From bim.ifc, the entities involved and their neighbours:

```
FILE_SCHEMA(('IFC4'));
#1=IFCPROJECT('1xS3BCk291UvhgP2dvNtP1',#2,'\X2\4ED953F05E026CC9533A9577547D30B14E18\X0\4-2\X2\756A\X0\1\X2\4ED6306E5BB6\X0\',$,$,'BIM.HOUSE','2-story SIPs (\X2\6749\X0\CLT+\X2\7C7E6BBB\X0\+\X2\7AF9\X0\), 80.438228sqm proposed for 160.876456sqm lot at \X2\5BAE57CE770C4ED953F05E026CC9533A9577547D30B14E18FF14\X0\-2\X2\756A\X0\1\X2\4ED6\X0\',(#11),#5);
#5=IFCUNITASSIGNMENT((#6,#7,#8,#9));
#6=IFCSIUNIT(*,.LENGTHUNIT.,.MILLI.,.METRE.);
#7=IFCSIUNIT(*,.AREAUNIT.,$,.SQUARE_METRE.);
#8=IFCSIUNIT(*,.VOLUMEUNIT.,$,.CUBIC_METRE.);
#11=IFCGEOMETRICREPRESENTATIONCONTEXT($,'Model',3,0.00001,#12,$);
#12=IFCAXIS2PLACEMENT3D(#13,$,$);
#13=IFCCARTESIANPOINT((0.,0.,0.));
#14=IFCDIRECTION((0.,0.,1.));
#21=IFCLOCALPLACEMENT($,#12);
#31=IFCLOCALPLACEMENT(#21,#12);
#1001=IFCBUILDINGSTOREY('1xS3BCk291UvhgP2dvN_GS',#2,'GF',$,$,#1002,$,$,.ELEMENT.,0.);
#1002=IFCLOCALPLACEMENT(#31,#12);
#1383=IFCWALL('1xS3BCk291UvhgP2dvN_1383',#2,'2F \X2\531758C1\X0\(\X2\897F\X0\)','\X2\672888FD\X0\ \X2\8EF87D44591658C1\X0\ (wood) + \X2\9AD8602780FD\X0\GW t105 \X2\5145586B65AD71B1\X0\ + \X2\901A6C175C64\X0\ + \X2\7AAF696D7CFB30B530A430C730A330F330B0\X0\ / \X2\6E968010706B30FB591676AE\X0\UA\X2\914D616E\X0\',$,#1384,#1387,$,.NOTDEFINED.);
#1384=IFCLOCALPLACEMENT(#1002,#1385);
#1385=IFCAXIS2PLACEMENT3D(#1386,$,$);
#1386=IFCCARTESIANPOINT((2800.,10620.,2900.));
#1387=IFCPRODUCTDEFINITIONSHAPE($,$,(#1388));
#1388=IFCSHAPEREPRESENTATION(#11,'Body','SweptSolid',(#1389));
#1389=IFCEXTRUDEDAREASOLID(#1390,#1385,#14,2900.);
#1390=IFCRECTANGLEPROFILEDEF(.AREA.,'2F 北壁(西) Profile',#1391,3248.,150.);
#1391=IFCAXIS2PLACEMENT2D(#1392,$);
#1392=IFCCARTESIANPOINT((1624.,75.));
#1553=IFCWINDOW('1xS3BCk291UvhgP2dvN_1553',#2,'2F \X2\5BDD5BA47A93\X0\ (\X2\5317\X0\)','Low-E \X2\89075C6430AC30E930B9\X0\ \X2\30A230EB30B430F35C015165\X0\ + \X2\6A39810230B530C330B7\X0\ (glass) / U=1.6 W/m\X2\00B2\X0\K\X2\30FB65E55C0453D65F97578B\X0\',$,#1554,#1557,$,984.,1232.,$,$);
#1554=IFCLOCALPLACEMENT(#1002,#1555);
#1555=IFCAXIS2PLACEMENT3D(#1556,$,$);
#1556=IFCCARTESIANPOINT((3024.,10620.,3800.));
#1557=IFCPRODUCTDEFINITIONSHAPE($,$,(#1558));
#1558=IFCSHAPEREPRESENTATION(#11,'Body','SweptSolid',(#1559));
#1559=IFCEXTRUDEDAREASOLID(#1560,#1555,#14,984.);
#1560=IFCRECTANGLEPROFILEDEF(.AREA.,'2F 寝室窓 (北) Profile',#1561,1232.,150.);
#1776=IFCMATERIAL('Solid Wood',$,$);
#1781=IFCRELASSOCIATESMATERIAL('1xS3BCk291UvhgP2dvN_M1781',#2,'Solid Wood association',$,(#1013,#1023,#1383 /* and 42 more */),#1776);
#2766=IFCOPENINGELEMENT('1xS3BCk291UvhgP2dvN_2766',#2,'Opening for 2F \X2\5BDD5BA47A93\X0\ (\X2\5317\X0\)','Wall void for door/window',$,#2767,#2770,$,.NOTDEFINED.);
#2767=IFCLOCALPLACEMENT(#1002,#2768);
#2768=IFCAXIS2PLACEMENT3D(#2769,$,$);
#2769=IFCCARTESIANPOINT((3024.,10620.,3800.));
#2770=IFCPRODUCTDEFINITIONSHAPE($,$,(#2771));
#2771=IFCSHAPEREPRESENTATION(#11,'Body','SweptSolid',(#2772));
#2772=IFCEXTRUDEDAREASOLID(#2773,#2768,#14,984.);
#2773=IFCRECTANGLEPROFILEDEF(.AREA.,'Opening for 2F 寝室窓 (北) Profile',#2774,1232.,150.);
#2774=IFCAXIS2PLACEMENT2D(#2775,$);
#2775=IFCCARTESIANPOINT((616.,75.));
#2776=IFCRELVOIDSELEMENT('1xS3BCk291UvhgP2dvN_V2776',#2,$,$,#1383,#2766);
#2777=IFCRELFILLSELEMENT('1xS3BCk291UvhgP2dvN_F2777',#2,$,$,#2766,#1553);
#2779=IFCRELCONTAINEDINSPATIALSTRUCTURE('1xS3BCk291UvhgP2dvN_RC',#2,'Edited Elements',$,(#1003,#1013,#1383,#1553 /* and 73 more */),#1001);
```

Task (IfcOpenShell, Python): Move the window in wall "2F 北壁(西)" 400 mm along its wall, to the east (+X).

```python
import ifcopenshell
import ifcopenshell.api.geometry
import ifcopenshell.util.placement

model = ifcopenshell.open("bim.ifc")

window = model.by_guid("1xS3BCk291UvhgP2dvN_1553")
opening = window.FillsVoids[0].RelatingOpeningElement
wall = opening.VoidsElements[0].RelatingBuildingElement

wall_matrix = ifcopenshell.util.placement.get_local_placement(wall.ObjectPlacement)
shift = wall_matrix[:3, 0] * 400.0
before = ifcopenshell.util.placement.get_local_placement(window.ObjectPlacement)[:3, 3].copy()

# The window is not placed relative to its opening, so move both.
for product in (opening, window):
    matrix = ifcopenshell.util.placement.get_local_placement(product.ObjectPlacement)
    matrix[:3, 3] += shift
    ifcopenshell.api.geometry.edit_object_placement(model, product=product, matrix=matrix, is_si=False)

after = ifcopenshell.util.placement.get_local_placement(window.ObjectPlacement)[:3, 3]
print("window moved by", (after - before).round(3) + 0.0)

model.write("bim_edited.ifc")
```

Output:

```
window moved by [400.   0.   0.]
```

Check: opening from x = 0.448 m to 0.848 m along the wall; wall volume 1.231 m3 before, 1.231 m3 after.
